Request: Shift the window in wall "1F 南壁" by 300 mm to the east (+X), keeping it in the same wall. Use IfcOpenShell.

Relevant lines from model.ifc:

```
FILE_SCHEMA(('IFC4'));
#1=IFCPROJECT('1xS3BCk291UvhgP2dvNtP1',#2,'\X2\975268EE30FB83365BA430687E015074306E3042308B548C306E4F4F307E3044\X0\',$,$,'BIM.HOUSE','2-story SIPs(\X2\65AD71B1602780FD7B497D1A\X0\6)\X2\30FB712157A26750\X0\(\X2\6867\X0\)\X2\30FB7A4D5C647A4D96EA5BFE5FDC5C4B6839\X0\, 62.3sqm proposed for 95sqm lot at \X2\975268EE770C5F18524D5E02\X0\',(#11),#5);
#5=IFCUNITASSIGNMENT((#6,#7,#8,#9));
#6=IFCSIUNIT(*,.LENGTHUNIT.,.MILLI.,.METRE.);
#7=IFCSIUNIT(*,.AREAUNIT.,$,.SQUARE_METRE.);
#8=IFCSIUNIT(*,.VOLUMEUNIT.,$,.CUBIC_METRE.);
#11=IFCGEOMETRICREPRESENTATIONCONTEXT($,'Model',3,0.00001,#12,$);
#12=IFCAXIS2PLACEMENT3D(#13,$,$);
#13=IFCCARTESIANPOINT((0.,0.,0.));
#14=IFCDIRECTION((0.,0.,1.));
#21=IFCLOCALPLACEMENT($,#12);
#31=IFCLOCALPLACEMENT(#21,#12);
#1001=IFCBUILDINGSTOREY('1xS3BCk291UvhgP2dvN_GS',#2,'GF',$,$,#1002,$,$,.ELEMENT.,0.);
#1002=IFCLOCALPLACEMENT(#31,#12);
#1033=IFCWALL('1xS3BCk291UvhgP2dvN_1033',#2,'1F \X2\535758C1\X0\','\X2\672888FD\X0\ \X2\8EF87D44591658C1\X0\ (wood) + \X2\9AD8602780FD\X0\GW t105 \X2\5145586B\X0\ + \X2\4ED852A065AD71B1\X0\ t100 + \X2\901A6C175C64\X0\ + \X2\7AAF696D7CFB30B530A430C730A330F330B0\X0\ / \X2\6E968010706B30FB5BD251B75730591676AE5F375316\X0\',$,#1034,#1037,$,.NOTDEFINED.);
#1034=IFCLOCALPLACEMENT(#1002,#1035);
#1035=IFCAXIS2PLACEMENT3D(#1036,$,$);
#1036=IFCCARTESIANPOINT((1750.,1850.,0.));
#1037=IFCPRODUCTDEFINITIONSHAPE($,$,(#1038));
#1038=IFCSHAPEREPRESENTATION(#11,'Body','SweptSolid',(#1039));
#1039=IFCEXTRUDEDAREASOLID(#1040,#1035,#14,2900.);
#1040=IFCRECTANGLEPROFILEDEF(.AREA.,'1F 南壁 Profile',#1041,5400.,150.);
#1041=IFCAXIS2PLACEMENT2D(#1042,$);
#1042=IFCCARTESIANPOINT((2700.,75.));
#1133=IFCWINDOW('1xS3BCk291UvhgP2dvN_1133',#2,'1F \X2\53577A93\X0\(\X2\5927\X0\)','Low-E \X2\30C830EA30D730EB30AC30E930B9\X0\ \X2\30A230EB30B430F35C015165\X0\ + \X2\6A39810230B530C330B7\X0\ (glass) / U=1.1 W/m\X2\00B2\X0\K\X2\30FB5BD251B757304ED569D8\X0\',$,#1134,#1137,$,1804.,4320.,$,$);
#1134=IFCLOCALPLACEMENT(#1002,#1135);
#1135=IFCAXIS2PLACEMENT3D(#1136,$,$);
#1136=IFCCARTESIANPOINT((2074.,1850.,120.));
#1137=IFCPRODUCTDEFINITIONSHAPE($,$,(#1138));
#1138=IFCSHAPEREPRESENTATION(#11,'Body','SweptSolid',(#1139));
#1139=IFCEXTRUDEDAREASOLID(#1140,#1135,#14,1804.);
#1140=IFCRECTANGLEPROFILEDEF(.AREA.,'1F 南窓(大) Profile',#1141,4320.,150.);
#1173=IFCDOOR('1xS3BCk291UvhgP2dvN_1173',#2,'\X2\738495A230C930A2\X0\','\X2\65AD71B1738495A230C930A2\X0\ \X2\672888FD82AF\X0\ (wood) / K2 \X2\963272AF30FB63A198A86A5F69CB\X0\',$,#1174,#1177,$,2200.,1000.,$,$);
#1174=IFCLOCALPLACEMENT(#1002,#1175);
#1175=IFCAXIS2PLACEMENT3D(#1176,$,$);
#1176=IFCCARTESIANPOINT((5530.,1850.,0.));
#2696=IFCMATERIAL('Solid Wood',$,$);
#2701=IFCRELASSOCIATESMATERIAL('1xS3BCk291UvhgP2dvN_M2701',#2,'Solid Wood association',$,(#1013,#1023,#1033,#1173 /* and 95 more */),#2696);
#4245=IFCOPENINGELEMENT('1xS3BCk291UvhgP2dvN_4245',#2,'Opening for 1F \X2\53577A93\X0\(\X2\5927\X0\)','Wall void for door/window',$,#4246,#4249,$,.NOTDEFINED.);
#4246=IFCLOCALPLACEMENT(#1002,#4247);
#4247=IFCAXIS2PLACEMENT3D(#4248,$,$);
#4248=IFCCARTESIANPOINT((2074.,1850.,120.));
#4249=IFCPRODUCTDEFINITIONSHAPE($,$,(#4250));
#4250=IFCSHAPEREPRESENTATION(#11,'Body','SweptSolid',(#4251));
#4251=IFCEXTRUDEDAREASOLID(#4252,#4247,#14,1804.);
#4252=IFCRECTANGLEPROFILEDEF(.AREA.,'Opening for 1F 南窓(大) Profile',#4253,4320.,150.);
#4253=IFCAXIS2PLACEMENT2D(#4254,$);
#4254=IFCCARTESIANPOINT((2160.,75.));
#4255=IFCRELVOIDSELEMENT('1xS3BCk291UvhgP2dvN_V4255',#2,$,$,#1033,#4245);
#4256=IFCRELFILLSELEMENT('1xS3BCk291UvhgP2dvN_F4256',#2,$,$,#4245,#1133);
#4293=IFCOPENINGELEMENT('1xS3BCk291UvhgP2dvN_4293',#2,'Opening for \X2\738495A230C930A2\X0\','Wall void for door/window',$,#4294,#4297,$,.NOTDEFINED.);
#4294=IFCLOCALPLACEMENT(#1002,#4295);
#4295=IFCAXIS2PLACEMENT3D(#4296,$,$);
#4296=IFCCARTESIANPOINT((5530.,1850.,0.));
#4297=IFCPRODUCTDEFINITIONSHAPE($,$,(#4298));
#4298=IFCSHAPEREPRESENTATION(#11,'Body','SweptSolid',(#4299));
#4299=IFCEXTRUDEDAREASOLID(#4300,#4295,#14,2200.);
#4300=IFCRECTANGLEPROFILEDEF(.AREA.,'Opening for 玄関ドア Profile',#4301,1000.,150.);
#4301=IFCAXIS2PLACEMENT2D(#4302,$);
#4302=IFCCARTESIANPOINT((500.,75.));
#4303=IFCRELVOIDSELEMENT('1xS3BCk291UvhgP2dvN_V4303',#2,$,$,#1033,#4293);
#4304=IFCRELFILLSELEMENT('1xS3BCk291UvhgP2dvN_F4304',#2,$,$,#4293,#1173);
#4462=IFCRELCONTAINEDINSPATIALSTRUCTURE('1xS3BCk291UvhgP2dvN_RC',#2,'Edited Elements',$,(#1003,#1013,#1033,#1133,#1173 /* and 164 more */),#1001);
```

```python
import ifcopenshell
import ifcopenshell.api.geometry
import ifcopenshell.util.placement
import ifcopenshell.util.unit

model = ifcopenshell.open("model.ifc")
unit_scale = ifcopenshell.util.unit.calculate_unit_scale(model)

window = model.by_guid("1xS3BCk291UvhgP2dvN_1133")
opening = window.FillsVoids[0].RelatingOpeningElement
wall = opening.VoidsElements[0].RelatingBuildingElement

wall_matrix = ifcopenshell.util.placement.get_local_placement(wall.ObjectPlacement)
shift = wall_matrix[:3, 0] * 0.3 / unit_scale
before = ifcopenshell.util.placement.get_local_placement(window.ObjectPlacement)[:3, 3].copy()

# The window is not placed relative to its opening, so move both.
for product in (opening, window):
    matrix = ifcopenshell.util.placement.get_local_placement(product.ObjectPlacement)
    matrix[:3, 3] += shift
    ifcopenshell.api.geometry.edit_object_placement(model, product=product, matrix=matrix, is_si=False)

after = ifcopenshell.util.placement.get_local_placement(window.ObjectPlacement)[:3, 3]
print("window moved by", (after - before).round(3) + 0.0)

model.write("model_updated.ifc")
```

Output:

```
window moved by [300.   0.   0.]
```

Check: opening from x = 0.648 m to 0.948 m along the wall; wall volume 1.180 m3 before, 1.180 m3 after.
